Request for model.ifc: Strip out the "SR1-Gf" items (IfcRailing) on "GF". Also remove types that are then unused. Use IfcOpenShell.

First a look at what the model holds.

```python
import ifcopenshell
import ifcopenshell.util.element

model = ifcopenshell.open("model.ifc")
print(model.schema)
storey = next(s for s in model.by_type("IfcBuildingStorey") if s.Name == "GF")
railings = [e for e in ifcopenshell.util.element.get_decomposition(storey) if e.is_a("IfcRailing")]
seen = {}
for e in railings:
    element_type = ifcopenshell.util.element.get_type(e)
    name = element_type.Name if element_type not in (None, e) else None
    seen[name] = seen.get(name, 0) + 1
for name, count in sorted(seen.items(), key=str):
    print(count, "x", name)
```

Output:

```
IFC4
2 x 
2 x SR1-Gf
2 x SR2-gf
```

```python
import ifcopenshell
import ifcopenshell.api.root
import ifcopenshell.util.element

model = ifcopenshell.open("model.ifc")

storey = next(s for s in model.by_type("IfcBuildingStorey") if s.Name == "GF")
railings = [e for e in ifcopenshell.util.element.get_decomposition(storey) if e.is_a("IfcRailing")]
targets = [e for e in railings if (t := ifcopenshell.util.element.get_type(e)) not in (None, e) and t.Name == "SR1-Gf"]
types = {ifcopenshell.util.element.get_type(e) for e in targets} - {None, *targets}

for e in targets:
    ifcopenshell.api.root.remove_product(model, product=e)
print(len(targets), "removed")

unused = [t for t in types if not ifcopenshell.util.element.get_types(t)]
for t in unused:
    ifcopenshell.api.root.remove_product(model, product=t)
print(len(unused), "unused types removed")

model.write("model-out.ifc")
```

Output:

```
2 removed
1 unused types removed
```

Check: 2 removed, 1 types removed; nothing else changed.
